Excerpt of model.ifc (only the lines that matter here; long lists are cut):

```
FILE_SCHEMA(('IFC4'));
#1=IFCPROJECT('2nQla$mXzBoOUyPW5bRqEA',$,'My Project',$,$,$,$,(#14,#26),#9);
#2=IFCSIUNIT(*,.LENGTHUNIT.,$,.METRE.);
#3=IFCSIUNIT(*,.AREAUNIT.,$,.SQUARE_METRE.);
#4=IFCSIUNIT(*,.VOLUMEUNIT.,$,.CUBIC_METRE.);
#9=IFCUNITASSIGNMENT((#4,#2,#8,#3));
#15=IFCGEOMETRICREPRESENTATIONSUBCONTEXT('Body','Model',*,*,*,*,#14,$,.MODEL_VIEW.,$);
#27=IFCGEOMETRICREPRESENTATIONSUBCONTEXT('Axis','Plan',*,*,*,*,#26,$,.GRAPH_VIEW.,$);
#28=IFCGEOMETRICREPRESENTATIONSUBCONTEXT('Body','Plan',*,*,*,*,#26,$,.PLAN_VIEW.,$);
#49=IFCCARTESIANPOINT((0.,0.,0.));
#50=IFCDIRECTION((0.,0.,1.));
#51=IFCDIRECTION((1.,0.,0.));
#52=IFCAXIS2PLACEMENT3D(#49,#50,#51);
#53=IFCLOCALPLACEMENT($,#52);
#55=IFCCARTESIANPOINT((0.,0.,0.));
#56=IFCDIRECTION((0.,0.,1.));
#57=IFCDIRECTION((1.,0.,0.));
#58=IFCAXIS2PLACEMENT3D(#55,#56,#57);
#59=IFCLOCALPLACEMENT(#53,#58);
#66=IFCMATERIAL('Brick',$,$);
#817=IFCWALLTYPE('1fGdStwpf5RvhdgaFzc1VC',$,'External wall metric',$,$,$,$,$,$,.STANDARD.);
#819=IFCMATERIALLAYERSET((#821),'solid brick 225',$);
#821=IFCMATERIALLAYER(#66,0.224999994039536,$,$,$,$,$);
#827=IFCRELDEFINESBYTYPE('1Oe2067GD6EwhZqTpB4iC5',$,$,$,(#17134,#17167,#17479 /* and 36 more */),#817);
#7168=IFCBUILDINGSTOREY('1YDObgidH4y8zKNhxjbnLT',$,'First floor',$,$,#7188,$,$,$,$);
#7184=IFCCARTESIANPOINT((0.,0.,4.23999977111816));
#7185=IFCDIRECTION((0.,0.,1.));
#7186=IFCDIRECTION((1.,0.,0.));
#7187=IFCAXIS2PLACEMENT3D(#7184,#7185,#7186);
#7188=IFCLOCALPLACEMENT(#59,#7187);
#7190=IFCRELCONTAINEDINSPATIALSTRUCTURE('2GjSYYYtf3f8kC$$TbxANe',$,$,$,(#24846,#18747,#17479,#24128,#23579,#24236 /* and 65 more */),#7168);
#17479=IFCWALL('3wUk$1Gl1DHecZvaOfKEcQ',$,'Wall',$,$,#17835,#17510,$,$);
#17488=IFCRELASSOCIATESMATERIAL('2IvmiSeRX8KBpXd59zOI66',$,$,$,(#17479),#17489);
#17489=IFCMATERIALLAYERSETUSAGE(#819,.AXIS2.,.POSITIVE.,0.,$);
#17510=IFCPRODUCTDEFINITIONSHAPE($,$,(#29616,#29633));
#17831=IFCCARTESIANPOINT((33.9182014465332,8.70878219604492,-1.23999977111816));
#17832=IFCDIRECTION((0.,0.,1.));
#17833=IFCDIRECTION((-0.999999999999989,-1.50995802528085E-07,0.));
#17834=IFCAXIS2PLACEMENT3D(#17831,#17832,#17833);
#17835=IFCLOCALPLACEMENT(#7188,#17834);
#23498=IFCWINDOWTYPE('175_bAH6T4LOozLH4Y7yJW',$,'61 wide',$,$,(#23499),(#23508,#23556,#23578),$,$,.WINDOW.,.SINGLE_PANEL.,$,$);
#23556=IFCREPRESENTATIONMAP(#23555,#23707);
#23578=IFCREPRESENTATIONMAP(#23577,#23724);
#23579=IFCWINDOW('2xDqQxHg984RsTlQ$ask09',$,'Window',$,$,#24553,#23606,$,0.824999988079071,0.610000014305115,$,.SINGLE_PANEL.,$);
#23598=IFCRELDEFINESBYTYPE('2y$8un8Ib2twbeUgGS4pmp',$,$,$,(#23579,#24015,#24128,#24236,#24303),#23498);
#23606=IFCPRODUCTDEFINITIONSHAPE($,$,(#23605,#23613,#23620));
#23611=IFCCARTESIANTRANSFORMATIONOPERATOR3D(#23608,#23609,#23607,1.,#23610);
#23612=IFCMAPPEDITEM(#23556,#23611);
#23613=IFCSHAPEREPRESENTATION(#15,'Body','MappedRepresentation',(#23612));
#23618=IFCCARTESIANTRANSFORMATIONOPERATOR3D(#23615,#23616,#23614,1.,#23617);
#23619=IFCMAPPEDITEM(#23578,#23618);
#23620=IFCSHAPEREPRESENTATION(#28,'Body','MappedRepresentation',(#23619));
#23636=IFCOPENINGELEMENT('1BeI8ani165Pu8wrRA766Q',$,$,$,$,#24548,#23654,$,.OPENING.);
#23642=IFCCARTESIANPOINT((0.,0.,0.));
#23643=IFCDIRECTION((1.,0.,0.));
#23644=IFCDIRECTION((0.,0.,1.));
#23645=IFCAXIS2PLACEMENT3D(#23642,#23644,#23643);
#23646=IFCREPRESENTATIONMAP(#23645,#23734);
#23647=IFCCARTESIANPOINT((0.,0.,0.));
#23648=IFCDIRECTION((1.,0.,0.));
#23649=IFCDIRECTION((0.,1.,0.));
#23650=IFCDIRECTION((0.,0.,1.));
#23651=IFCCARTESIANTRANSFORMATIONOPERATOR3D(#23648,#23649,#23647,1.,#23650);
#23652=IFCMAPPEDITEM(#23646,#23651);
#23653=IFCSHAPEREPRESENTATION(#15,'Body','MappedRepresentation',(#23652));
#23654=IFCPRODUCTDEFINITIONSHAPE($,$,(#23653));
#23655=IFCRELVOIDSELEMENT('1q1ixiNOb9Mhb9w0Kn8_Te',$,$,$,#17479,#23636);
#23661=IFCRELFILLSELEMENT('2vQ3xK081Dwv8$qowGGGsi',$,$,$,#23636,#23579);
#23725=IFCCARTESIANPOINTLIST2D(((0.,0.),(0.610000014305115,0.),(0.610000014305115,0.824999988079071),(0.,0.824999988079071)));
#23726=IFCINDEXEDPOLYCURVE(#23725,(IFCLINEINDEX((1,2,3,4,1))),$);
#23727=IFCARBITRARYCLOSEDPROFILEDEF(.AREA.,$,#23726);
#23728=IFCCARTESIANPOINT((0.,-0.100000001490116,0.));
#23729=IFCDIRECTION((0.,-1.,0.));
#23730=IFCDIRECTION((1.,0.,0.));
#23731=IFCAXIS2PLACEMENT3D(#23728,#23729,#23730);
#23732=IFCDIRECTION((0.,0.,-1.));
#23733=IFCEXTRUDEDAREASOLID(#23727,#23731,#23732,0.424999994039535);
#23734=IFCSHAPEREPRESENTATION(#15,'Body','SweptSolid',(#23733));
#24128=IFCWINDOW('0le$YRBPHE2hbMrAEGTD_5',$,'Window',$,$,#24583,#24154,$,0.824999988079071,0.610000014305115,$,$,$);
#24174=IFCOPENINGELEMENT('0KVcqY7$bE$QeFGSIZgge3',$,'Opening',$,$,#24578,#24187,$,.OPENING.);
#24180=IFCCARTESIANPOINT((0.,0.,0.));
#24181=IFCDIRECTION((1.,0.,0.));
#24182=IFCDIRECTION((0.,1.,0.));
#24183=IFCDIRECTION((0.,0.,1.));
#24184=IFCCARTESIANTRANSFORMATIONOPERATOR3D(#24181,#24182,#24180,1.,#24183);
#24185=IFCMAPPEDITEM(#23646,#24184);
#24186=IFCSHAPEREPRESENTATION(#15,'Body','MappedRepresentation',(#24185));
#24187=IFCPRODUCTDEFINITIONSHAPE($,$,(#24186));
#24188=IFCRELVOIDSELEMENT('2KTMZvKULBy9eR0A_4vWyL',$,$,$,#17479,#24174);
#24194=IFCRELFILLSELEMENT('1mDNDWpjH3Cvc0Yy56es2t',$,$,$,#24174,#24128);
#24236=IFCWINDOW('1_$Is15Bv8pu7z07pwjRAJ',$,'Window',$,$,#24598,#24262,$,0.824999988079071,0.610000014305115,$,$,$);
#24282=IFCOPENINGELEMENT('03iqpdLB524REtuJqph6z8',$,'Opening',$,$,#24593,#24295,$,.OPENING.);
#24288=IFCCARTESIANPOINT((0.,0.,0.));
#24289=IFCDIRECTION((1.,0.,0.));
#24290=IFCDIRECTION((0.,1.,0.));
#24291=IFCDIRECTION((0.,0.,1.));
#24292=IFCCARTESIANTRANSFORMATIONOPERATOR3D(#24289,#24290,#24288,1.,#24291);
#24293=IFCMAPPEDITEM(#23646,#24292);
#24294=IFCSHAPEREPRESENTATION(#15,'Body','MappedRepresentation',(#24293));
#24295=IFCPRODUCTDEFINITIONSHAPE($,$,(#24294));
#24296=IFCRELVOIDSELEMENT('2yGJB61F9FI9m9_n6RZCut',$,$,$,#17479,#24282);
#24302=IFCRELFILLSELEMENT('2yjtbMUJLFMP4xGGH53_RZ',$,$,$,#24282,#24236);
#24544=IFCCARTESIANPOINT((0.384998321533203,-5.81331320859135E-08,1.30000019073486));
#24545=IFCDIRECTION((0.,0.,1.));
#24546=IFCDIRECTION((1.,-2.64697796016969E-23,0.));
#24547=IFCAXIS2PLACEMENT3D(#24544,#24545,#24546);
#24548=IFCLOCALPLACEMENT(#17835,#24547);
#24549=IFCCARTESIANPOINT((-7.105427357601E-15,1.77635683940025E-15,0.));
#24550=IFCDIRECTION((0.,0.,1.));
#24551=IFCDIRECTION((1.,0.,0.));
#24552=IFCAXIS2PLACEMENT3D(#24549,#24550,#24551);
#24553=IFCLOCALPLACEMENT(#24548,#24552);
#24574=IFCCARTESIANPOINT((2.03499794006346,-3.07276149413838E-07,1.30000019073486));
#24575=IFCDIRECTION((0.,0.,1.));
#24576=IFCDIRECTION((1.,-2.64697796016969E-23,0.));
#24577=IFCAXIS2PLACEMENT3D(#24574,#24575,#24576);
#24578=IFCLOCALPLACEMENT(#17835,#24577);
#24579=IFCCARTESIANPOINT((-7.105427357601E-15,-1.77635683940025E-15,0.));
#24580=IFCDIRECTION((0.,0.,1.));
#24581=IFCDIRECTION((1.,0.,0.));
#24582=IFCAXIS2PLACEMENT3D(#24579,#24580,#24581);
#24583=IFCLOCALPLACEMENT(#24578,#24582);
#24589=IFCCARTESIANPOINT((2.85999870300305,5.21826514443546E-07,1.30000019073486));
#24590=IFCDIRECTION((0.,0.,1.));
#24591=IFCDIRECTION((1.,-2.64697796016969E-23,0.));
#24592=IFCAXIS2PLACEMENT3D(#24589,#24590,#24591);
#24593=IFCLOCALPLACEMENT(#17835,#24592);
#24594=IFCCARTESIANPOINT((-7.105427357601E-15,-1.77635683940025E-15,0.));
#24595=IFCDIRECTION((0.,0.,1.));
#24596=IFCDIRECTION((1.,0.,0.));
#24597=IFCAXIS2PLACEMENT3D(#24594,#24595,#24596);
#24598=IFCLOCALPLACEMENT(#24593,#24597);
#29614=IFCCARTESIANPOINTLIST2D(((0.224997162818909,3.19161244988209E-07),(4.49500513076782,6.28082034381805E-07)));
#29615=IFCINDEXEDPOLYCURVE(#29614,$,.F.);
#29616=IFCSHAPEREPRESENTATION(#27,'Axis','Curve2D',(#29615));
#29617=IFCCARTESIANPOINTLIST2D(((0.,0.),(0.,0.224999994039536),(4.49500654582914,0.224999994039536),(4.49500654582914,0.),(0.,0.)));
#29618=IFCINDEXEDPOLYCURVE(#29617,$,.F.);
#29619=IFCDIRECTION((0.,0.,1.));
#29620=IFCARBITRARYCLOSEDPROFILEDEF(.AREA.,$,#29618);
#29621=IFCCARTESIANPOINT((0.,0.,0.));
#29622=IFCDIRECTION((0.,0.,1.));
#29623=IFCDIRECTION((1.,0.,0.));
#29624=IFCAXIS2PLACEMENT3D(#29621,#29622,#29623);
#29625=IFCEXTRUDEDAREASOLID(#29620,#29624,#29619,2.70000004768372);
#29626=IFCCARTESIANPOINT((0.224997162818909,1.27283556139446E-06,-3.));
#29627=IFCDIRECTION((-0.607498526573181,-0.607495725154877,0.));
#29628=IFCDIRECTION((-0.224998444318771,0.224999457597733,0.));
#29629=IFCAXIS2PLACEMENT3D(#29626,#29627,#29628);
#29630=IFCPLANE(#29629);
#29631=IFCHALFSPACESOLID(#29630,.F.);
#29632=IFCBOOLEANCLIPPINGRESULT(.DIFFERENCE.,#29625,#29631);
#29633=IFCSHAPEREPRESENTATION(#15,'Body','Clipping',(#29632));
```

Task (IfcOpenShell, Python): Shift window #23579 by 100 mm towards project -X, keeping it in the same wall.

```python
import ifcopenshell
import ifcopenshell.api.geometry
import ifcopenshell.util.placement
import ifcopenshell.util.unit

model = ifcopenshell.open("model.ifc")
unit_scale = ifcopenshell.util.unit.calculate_unit_scale(model)

window = model.by_guid("2xDqQxHg984RsTlQ$ask09")
opening = window.FillsVoids[0].RelatingOpeningElement
wall = opening.VoidsElements[0].RelatingBuildingElement

wall_matrix = ifcopenshell.util.placement.get_local_placement(wall.ObjectPlacement)
shift = wall_matrix[:3, 0] * 0.1 / unit_scale
before = ifcopenshell.util.placement.get_local_placement(window.ObjectPlacement)[:3, 3].copy()

# The window is placed relative to its opening, so it follows when the opening moves.
matrix = ifcopenshell.util.placement.get_local_placement(opening.ObjectPlacement)
matrix[:3, 3] += shift
ifcopenshell.api.geometry.edit_object_placement(
    model, product=opening, matrix=matrix, is_si=False, should_transform_children=True
)

after = ifcopenshell.util.placement.get_local_placement(window.ObjectPlacement)[:3, 3]
print("window moved by", (after - before).round(3) + 0.0)

model.write("model_rev.ifc")
```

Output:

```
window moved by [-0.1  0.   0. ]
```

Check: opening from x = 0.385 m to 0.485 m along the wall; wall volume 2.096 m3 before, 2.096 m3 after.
